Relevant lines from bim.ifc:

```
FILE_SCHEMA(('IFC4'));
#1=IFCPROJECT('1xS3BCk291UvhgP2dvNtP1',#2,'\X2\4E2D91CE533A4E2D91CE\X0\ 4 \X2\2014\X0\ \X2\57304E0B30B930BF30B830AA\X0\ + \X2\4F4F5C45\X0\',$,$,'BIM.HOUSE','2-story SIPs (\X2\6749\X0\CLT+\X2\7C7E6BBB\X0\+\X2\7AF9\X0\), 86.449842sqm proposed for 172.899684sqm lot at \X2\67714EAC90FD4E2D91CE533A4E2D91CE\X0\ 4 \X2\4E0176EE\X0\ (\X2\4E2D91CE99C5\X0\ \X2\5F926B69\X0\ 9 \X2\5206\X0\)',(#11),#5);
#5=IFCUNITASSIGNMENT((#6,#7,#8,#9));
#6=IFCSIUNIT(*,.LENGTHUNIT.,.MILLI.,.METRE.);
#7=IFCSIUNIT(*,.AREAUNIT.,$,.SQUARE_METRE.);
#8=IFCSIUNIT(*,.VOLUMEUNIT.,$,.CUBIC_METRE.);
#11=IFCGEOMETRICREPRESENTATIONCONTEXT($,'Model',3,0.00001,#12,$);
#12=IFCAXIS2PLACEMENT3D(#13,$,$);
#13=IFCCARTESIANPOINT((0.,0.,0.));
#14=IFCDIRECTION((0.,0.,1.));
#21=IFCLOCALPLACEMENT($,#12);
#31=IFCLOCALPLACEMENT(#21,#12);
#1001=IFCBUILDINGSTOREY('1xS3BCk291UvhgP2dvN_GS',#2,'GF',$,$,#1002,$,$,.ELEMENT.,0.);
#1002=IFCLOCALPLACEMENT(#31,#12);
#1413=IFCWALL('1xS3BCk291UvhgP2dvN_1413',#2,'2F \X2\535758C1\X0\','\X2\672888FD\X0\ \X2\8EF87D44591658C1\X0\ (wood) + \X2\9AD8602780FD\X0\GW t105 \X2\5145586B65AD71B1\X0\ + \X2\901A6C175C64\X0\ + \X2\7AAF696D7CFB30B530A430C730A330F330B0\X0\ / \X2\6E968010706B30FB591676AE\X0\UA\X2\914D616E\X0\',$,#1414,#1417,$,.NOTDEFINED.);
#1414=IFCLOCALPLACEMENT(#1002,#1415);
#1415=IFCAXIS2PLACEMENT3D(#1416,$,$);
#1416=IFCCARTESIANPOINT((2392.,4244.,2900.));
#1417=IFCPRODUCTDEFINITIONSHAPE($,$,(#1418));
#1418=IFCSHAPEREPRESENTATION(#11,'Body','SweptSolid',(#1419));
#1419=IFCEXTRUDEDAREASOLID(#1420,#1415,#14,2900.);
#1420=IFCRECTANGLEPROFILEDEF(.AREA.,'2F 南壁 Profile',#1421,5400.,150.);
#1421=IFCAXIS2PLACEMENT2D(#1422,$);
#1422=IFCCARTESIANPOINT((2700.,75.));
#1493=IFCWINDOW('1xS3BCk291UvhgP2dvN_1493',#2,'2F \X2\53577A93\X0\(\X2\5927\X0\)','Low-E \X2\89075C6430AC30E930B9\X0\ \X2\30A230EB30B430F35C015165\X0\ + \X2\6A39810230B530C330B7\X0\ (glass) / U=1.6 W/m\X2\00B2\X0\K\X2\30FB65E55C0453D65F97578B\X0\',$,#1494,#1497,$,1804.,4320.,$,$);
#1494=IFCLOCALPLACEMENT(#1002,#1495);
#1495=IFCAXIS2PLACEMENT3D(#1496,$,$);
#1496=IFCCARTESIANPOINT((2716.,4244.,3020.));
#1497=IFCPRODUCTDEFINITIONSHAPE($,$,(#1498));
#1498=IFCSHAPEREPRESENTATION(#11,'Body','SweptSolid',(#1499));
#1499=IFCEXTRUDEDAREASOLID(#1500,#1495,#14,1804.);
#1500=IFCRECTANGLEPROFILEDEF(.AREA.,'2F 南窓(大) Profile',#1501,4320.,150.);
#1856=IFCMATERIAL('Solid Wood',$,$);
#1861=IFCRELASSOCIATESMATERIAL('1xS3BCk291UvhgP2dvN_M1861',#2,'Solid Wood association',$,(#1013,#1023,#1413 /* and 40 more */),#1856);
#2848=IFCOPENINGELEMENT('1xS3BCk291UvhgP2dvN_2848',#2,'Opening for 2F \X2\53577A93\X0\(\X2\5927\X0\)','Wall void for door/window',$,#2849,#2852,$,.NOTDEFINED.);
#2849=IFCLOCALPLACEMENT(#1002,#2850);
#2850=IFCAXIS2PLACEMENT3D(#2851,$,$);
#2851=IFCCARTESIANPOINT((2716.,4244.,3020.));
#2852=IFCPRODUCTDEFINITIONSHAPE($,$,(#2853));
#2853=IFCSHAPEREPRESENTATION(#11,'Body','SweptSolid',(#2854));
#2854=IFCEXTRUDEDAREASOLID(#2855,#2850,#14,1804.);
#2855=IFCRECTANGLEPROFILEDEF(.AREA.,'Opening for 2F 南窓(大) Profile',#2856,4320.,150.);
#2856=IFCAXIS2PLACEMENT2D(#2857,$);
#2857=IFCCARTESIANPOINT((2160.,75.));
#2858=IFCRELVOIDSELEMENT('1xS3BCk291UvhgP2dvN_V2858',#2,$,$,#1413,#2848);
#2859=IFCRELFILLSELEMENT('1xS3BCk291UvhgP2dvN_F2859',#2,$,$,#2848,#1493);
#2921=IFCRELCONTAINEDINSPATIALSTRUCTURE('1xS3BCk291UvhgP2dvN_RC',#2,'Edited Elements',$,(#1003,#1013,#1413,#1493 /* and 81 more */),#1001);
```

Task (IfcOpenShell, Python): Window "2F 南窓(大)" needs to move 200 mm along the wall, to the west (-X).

```python
import ifcopenshell
import ifcopenshell.api.geometry
import ifcopenshell.util.placement

model = ifcopenshell.open("bim.ifc")

window = model.by_id(1493)
opening = window.FillsVoids[0].RelatingOpeningElement
wall = opening.VoidsElements[0].RelatingBuildingElement

wall_matrix = ifcopenshell.util.placement.get_local_placement(wall.ObjectPlacement)
shift = wall_matrix[:3, 0] * -200.0
before = ifcopenshell.util.placement.get_local_placement(window.ObjectPlacement)[:3, 3].copy()

# The window is not placed relative to its opening, so move both.
for product in (opening, window):
    matrix = ifcopenshell.util.placement.get_local_placement(product.ObjectPlacement)
    matrix[:3, 3] += shift
    ifcopenshell.api.geometry.edit_object_placement(model, product=product, matrix=matrix, is_si=False)

after = ifcopenshell.util.placement.get_local_placement(window.ObjectPlacement)[:3, 3]
print("window moved by", (after - before).round(3) + 0.0)

model.write("bim_v2.ifc")
```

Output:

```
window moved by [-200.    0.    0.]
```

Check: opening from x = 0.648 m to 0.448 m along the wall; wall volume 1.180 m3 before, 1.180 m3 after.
